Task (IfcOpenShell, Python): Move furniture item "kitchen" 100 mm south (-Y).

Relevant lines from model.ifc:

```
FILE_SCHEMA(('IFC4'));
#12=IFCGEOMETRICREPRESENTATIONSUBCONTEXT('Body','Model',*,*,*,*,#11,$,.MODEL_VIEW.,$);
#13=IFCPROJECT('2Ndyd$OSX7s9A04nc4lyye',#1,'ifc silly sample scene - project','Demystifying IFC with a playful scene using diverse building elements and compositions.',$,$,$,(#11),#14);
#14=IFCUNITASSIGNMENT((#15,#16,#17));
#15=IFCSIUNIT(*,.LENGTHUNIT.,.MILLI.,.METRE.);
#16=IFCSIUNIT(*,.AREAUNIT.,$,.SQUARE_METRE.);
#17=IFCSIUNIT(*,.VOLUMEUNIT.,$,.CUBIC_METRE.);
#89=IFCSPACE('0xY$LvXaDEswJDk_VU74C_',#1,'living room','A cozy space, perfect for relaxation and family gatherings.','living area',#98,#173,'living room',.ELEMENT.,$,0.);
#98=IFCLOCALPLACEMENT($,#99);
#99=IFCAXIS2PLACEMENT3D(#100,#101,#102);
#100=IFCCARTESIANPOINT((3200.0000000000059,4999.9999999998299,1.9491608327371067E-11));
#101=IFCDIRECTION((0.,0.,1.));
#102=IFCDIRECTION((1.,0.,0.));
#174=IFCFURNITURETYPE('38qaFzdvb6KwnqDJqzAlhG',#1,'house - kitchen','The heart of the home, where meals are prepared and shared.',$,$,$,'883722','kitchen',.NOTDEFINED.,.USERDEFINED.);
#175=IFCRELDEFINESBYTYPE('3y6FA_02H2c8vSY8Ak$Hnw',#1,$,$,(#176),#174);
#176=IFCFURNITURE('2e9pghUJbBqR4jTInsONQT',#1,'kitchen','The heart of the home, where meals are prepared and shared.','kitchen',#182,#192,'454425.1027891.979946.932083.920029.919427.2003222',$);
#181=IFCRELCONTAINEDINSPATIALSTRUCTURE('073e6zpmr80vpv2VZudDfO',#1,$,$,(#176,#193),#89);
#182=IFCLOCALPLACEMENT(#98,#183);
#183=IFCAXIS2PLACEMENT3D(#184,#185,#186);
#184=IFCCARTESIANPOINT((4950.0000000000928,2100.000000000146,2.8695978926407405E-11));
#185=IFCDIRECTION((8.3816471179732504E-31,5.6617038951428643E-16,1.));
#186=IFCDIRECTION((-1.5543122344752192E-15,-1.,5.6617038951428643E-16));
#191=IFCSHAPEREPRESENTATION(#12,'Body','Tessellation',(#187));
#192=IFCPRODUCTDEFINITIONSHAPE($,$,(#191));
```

```python
import ifcopenshell
import ifcopenshell.api.geometry
import ifcopenshell.util.placement
import ifcopenshell.util.unit

model = ifcopenshell.open("model.ifc")
unit_scale = ifcopenshell.util.unit.calculate_unit_scale(model)

item = model.by_id(176)
matrix = ifcopenshell.util.placement.get_local_placement(item.ObjectPlacement)
matrix[1, 3] -= 0.1 / unit_scale
ifcopenshell.api.geometry.edit_object_placement(model, product=item, matrix=matrix, is_si=False)

print(ifcopenshell.util.placement.get_local_placement(item.ObjectPlacement).round(3) + 0.0)

model.write("model_updated.ifc")
```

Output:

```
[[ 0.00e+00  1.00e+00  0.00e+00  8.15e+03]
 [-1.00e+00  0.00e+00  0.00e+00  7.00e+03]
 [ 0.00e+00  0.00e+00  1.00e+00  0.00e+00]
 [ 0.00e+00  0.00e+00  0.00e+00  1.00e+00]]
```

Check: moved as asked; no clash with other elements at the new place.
